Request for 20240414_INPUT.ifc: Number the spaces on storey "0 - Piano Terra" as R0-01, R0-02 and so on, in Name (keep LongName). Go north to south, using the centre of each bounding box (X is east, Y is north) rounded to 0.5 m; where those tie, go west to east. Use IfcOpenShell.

First a look at what the model holds.

```python
import ifcopenshell
import ifcopenshell.util.element
import ifcopenshell.util.placement

model = ifcopenshell.open("20240414_INPUT.ifc")
print(model.schema)
storey = next(s for s in model.by_type("IfcBuildingStorey") if s.Name == "0 - Piano Terra")
spaces = [e for e in ifcopenshell.util.element.get_decomposition(storey) if e.is_a("IfcSpace")]
for e in sorted(spaces, key=lambda e: e.id()):
    origin = ifcopenshell.util.placement.get_local_placement(e.ObjectPlacement)[:3, 3]
    print(e.id(), e.Name, e.LongName, origin.round(2) + 0.0, sep=" | ")
```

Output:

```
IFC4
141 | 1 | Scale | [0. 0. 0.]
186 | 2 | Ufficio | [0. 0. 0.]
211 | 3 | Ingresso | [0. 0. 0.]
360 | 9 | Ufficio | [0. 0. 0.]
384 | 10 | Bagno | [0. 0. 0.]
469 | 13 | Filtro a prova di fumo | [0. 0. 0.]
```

```python
import ifcopenshell
import ifcopenshell.geom
import ifcopenshell.util.element
import ifcopenshell.util.shape

model = ifcopenshell.open("20240414_INPUT.ifc")
settings = ifcopenshell.geom.settings()
settings.set("use-world-coords", True)


def centre(element):
    shape = ifcopenshell.geom.create_shape(settings, element)
    return ifcopenshell.util.shape.get_bbox_centroid(shape.geometry)


storey = next(s for s in model.by_type("IfcBuildingStorey") if s.Name == "0 - Piano Terra")
spaces = [e for e in ifcopenshell.util.element.get_decomposition(storey) if e.is_a("IfcSpace")]

# Insertion points can sit at a corner or the storey origin, so sort by the geometry (in metres).
centres = {e: centre(e) for e in spaces}
spaces.sort(key=lambda e: (-round(centres[e][1] / 0.5), centres[e][0]))

for i, e in enumerate(spaces, start=1):
    number = f"R0-{i:02d}"
    e.Name = number
    print(e.id(), number)

model.write("20240414_INPUT_v2.ifc")
```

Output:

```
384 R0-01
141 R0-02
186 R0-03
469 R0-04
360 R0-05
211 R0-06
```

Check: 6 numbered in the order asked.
